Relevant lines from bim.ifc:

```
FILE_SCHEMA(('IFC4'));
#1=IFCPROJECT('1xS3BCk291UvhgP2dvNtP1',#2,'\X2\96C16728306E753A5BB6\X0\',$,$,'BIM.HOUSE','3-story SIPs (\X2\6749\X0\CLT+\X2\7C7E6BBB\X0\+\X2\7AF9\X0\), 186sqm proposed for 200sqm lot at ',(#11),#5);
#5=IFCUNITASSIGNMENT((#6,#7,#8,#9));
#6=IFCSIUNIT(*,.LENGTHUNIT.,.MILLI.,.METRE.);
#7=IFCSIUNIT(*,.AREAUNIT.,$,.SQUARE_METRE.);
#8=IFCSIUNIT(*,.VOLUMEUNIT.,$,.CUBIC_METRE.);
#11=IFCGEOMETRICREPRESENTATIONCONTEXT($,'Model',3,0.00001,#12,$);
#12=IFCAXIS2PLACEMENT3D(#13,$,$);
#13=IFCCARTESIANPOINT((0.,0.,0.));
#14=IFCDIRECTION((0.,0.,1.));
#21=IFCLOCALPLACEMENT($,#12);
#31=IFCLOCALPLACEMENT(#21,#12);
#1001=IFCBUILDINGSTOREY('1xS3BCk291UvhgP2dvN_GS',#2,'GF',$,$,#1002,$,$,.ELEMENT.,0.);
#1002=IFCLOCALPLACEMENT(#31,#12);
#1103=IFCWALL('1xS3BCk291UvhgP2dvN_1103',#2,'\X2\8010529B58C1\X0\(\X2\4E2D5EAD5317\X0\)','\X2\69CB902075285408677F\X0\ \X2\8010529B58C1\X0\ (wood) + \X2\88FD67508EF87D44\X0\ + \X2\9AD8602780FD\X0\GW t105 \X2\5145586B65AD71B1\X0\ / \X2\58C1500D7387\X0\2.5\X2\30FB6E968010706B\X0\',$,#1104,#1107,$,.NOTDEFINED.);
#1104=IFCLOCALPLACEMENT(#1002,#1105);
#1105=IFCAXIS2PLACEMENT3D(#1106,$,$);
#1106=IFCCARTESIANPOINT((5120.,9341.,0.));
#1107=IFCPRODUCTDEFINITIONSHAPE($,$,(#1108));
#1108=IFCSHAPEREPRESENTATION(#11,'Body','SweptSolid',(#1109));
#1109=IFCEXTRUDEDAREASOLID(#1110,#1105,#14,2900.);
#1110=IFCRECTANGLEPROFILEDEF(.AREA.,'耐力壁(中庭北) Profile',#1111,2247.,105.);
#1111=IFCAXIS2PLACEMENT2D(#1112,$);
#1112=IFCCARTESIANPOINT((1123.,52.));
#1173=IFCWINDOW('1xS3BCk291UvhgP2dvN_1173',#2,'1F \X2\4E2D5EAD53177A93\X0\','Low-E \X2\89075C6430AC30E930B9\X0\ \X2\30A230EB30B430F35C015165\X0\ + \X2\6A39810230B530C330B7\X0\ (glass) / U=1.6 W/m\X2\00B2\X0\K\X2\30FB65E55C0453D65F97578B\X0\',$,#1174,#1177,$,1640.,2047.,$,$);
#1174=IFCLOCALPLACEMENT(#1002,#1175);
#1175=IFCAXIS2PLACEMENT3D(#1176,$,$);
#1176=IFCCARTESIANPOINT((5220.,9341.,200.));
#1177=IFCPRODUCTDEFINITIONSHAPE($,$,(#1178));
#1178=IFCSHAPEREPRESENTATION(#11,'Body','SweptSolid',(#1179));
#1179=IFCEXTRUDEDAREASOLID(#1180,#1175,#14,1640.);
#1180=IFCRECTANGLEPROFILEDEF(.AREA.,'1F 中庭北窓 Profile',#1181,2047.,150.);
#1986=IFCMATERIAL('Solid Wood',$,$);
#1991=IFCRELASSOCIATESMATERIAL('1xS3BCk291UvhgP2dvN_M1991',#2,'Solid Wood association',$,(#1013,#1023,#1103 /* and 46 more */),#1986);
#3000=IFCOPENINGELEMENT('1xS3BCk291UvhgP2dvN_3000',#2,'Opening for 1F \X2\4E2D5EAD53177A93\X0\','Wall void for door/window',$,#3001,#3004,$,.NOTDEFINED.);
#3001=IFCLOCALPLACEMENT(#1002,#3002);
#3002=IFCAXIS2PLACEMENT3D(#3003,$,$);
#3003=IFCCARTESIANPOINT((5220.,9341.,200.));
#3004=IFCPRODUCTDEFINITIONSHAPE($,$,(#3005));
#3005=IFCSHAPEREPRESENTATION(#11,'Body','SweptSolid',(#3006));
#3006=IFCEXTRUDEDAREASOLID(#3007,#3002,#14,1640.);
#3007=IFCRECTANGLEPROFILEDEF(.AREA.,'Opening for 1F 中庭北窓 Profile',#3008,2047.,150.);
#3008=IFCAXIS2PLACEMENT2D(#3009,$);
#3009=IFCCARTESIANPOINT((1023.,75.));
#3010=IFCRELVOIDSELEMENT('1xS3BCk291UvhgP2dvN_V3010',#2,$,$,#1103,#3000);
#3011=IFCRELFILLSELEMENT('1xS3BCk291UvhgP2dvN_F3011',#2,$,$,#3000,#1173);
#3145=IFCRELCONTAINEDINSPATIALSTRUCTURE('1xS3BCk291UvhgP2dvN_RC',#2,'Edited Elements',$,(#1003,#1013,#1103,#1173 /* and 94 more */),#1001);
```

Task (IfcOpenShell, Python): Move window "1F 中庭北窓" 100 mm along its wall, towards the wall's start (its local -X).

```python
import ifcopenshell
import ifcopenshell.api.geometry
import ifcopenshell.util.placement
import ifcopenshell.util.unit

model = ifcopenshell.open("bim.ifc")
unit_scale = ifcopenshell.util.unit.calculate_unit_scale(model)

window = model.by_guid("1xS3BCk291UvhgP2dvN_1173")
opening = window.FillsVoids[0].RelatingOpeningElement
wall = opening.VoidsElements[0].RelatingBuildingElement

wall_matrix = ifcopenshell.util.placement.get_local_placement(wall.ObjectPlacement)
shift = wall_matrix[:3, 0] * -0.1 / unit_scale
before = ifcopenshell.util.placement.get_local_placement(window.ObjectPlacement)[:3, 3].copy()

# The window is not placed relative to its opening, so move both.
for product in (opening, window):
    matrix = ifcopenshell.util.placement.get_local_placement(product.ObjectPlacement)
    matrix[:3, 3] += shift
    ifcopenshell.api.geometry.edit_object_placement(model, product=product, matrix=matrix, is_si=False)

after = ifcopenshell.util.placement.get_local_placement(window.ObjectPlacement)[:3, 3]
print("window moved by", (after - before).round(3) + 0.0)

model.write("bim_edited.ifc")
```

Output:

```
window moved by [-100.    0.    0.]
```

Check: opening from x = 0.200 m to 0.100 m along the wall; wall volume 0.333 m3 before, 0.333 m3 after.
